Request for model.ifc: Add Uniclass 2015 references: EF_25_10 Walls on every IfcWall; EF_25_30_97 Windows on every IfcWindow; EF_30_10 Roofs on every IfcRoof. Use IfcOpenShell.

First a look at what the model holds.

```python
import ifcopenshell

model = ifcopenshell.open("model.ifc")
print(model.schema)
print("classifications:", [c.Name for c in model.by_type("IfcClassification")])
for ifc_class in ("IfcDoor", "IfcRoof", "IfcStair", "IfcWall", "IfcWindow"):
    print(ifc_class, len(model.by_type(ifc_class)))
```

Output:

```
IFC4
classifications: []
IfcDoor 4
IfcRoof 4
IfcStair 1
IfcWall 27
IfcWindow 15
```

```python
import ifcopenshell
import ifcopenshell.api.classification

model = ifcopenshell.open("model.ifc")

system = ifcopenshell.api.classification.add_classification(model, classification="Uniclass 2015")

codes = {
    "IfcWall": ("EF_25_10", "Walls"),
    "IfcWindow": ("EF_25_30_97", "Windows"),
    "IfcRoof": ("EF_30_10", "Roofs"),
}
for ifc_class, (code, name) in codes.items():
    products = model.by_type(ifc_class)
    ifcopenshell.api.classification.add_reference(
        model, products=products, classification=system, identification=code, name=name
    )
    print(code, len(products))

model.write("model_edited.ifc")
```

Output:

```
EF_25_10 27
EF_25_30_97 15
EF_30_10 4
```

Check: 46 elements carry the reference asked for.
